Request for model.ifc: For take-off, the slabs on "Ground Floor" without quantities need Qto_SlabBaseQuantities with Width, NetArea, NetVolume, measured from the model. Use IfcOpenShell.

First a look at what the model holds.

```python
import ifcopenshell
import ifcopenshell.util.element
import ifcopenshell.util.unit

model = ifcopenshell.open("model.ifc")
print(model.schema)
for unit_type in ("LENGTHUNIT", "AREAUNIT", "VOLUMEUNIT"):
    print(unit_type, ifcopenshell.util.unit.calculate_unit_scale(model, unit_type))
storey = next(s for s in model.by_type("IfcBuildingStorey") if s.Name == "Ground Floor")
slabs = [e for e in ifcopenshell.util.element.get_decomposition(storey) if e.is_a("IfcSlab")]
for e in sorted(slabs, key=lambda e: e.id()):
    print(e.id(), e.is_a(), e.Name, list(ifcopenshell.util.element.get_psets(e, qtos_only=True)), sep=" | ")
```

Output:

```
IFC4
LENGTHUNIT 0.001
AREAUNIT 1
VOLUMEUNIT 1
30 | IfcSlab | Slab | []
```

```python
import ifcopenshell
import ifcopenshell.api.pset
import ifcopenshell.geom
import ifcopenshell.util.element
import ifcopenshell.util.shape
import ifcopenshell.util.unit

model = ifcopenshell.open("model.ifc")
unit_scale = ifcopenshell.util.unit.calculate_unit_scale(model)
area_scale = ifcopenshell.util.unit.calculate_unit_scale(model, "AREAUNIT")
volume_scale = ifcopenshell.util.unit.calculate_unit_scale(model, "VOLUMEUNIT")
settings = ifcopenshell.geom.settings()

storey = next(s for s in model.by_type("IfcBuildingStorey") if s.Name == "Ground Floor")
slabs = [e for e in ifcopenshell.util.element.get_decomposition(storey) if e.is_a("IfcSlab")]

for e in sorted(slabs, key=lambda e: e.id()):
    if ifcopenshell.util.element.get_psets(e, qtos_only=True, should_inherit=False):
        continue
    # Geometry comes back in metres, in the element's own axes.
    shape = ifcopenshell.geom.create_shape(settings, e)
    values = {
        "Width": ifcopenshell.util.shape.get_z(shape.geometry) / unit_scale,
        "NetArea": ifcopenshell.util.shape.get_footprint_area(shape.geometry) / area_scale,
        "NetVolume": ifcopenshell.util.shape.get_volume(shape.geometry) / volume_scale,
    }
    qto = ifcopenshell.api.pset.add_qto(model, product=e, name="Qto_SlabBaseQuantities")
    ifcopenshell.api.pset.edit_qto(model, qto=qto, properties=values)
    print(e.id(), {k: round(v, 3) for k, v in values.items()})

model.write("model_rev.ifc")
```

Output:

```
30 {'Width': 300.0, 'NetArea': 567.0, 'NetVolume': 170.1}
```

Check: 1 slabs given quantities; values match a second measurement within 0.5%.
